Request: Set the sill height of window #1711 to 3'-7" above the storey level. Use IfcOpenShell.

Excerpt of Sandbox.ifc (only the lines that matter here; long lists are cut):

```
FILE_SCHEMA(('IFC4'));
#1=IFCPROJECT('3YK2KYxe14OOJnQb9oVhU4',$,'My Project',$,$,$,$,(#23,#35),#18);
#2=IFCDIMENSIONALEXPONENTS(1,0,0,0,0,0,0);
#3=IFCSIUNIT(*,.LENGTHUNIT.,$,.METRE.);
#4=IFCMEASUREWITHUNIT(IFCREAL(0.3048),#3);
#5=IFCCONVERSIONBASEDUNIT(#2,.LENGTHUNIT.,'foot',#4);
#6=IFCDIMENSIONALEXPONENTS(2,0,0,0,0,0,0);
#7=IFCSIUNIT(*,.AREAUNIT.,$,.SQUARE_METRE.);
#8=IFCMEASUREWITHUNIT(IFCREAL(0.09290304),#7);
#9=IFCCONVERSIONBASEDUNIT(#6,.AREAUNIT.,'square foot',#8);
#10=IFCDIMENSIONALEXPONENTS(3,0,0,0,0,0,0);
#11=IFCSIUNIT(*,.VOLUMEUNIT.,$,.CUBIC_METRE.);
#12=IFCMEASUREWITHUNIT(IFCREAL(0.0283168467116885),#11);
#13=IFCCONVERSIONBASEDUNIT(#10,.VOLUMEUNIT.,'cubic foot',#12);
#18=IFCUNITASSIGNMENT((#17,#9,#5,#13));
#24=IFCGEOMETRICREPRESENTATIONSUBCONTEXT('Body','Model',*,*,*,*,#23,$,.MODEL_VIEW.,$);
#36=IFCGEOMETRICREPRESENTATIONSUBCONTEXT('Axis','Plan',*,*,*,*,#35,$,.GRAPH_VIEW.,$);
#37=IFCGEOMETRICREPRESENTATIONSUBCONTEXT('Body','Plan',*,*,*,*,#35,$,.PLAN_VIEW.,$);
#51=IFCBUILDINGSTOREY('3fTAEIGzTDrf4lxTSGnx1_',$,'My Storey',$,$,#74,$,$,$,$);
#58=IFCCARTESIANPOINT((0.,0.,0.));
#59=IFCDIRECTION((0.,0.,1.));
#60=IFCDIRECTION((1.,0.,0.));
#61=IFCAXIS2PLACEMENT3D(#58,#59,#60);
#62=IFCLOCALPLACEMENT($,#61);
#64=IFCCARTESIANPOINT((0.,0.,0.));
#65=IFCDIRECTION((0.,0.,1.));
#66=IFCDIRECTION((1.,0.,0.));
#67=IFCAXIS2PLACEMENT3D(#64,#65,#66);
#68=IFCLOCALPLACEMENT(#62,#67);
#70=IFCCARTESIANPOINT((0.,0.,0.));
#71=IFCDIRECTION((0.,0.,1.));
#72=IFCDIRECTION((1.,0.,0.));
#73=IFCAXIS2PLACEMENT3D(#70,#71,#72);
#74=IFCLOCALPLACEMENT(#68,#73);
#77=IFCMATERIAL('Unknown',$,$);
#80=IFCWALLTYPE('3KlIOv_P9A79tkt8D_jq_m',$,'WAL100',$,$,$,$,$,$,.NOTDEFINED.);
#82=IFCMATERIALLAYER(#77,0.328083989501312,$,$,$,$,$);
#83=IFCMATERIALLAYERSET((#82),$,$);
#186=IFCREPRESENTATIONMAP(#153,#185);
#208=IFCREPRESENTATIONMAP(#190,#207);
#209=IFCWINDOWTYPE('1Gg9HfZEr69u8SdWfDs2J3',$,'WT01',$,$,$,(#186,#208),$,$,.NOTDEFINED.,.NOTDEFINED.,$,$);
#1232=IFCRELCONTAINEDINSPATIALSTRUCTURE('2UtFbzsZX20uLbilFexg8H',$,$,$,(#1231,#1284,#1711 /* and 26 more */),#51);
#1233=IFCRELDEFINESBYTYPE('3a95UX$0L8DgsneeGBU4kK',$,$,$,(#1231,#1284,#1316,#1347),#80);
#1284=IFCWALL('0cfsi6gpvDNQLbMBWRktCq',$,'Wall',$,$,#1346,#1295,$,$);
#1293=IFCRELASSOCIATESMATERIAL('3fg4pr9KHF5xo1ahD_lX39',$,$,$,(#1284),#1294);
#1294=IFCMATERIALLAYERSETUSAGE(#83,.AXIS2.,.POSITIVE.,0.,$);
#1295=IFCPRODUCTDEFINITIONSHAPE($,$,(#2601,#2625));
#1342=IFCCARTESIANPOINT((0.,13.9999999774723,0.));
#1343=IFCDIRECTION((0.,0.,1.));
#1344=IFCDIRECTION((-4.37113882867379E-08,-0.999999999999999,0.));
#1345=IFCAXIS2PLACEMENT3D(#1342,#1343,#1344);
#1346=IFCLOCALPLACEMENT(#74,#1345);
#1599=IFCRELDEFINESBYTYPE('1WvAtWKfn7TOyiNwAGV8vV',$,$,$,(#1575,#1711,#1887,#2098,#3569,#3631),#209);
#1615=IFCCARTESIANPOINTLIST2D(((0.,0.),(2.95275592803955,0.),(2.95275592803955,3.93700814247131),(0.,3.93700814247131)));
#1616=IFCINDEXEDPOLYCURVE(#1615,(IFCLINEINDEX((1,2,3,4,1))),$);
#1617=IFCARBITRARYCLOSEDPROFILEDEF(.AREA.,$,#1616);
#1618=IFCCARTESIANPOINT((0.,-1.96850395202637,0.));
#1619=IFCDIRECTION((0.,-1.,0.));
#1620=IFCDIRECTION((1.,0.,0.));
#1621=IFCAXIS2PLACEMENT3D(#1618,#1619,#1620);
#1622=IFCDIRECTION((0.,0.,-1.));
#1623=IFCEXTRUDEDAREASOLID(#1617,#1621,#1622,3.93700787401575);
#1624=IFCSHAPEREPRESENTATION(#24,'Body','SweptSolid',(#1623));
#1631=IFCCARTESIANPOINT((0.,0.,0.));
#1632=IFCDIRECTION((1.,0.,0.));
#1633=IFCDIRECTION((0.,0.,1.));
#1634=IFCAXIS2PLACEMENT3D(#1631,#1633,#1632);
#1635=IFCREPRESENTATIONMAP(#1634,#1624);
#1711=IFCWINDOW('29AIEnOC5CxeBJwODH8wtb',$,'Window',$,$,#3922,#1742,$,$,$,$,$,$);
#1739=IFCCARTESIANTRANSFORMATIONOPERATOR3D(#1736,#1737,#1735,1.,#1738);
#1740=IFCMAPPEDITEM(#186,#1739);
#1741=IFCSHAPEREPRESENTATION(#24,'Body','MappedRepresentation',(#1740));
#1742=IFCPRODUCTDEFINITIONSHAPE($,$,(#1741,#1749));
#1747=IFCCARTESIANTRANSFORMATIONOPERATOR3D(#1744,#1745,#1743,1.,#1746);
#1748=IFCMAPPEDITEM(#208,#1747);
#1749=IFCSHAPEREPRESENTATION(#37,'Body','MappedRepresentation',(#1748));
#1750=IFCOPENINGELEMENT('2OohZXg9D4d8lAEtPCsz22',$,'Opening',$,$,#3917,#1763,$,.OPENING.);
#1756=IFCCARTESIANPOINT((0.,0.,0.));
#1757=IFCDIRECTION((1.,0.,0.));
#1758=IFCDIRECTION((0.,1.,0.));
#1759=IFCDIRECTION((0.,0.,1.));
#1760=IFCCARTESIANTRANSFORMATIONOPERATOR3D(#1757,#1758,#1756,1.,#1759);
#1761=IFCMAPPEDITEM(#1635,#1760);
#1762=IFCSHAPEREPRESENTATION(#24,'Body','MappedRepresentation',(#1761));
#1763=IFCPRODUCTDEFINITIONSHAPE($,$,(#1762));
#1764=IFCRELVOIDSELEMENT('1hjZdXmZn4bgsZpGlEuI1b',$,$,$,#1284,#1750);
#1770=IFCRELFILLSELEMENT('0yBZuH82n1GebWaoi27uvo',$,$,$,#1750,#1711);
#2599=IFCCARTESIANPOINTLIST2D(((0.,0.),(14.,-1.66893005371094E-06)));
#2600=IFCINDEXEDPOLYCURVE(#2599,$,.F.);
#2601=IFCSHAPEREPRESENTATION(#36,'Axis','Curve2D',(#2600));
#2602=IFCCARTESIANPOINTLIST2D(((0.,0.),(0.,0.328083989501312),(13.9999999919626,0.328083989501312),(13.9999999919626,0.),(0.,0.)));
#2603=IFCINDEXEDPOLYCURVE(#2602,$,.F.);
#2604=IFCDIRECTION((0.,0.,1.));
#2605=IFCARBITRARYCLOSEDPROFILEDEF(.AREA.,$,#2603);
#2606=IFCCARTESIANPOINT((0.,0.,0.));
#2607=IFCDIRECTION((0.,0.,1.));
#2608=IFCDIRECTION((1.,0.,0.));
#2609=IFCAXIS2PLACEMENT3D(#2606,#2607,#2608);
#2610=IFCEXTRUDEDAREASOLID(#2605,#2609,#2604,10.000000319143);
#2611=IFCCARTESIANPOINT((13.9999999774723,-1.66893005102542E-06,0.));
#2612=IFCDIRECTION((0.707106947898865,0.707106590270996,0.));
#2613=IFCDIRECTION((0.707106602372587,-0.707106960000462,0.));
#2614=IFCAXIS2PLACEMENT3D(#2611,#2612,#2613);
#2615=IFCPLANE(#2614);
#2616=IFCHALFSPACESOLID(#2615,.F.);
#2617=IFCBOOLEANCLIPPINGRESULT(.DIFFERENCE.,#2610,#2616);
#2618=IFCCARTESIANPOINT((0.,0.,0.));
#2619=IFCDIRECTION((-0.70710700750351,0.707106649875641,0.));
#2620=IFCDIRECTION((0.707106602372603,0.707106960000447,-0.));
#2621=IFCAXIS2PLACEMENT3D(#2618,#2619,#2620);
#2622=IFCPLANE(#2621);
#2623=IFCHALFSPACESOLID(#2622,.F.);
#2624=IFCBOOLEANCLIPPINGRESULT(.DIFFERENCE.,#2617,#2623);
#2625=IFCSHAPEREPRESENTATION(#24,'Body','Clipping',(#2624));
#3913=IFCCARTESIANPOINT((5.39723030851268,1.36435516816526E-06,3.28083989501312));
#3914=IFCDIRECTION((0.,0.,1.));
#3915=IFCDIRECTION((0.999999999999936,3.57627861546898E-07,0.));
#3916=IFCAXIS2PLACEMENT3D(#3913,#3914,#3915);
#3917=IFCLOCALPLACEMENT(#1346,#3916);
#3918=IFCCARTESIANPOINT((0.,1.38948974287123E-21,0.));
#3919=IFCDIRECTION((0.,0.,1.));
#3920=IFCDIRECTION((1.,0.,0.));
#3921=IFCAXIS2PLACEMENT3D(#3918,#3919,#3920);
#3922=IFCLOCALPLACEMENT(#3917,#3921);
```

```python
import numpy as np
import ifcopenshell
import ifcopenshell.api.geometry
import ifcopenshell.geom
import ifcopenshell.util.element
import ifcopenshell.util.placement
import ifcopenshell.util.shape
import ifcopenshell.util.unit

model = ifcopenshell.open("Sandbox.ifc")
unit_scale = ifcopenshell.util.unit.calculate_unit_scale(model)

window = model.by_guid("29AIEnOC5CxeBJwODH8wtb")
opening = window.FillsVoids[0].RelatingOpeningElement
storey = ifcopenshell.util.element.get_container(window, ifc_class="IfcBuildingStorey")
level = ifcopenshell.util.placement.get_local_placement(storey.ObjectPlacement)[2, 3]

# The opening's origin need not be at the sill, so measure its lowest point.
shape = ifcopenshell.geom.create_shape(ifcopenshell.geom.settings(), opening)
bottom = ifcopenshell.util.shape.get_shape_bottom_elevation(shape, shape.geometry) / unit_scale
dz = level + 43 * 0.0254 / unit_scale - bottom

shift = np.array([0.0, 0.0, dz])
# The window is placed relative to its opening, so it follows when the opening moves.
matrix = ifcopenshell.util.placement.get_local_placement(opening.ObjectPlacement)
matrix[:3, 3] += shift
ifcopenshell.api.geometry.edit_object_placement(
    model, product=opening, matrix=matrix, is_si=False, should_transform_children=True
)

print(f"moved by {dz * unit_scale:+.3f} m")

model.write("Sandbox_v2.ifc")
```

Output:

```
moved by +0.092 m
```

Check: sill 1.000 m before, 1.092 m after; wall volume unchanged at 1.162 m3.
